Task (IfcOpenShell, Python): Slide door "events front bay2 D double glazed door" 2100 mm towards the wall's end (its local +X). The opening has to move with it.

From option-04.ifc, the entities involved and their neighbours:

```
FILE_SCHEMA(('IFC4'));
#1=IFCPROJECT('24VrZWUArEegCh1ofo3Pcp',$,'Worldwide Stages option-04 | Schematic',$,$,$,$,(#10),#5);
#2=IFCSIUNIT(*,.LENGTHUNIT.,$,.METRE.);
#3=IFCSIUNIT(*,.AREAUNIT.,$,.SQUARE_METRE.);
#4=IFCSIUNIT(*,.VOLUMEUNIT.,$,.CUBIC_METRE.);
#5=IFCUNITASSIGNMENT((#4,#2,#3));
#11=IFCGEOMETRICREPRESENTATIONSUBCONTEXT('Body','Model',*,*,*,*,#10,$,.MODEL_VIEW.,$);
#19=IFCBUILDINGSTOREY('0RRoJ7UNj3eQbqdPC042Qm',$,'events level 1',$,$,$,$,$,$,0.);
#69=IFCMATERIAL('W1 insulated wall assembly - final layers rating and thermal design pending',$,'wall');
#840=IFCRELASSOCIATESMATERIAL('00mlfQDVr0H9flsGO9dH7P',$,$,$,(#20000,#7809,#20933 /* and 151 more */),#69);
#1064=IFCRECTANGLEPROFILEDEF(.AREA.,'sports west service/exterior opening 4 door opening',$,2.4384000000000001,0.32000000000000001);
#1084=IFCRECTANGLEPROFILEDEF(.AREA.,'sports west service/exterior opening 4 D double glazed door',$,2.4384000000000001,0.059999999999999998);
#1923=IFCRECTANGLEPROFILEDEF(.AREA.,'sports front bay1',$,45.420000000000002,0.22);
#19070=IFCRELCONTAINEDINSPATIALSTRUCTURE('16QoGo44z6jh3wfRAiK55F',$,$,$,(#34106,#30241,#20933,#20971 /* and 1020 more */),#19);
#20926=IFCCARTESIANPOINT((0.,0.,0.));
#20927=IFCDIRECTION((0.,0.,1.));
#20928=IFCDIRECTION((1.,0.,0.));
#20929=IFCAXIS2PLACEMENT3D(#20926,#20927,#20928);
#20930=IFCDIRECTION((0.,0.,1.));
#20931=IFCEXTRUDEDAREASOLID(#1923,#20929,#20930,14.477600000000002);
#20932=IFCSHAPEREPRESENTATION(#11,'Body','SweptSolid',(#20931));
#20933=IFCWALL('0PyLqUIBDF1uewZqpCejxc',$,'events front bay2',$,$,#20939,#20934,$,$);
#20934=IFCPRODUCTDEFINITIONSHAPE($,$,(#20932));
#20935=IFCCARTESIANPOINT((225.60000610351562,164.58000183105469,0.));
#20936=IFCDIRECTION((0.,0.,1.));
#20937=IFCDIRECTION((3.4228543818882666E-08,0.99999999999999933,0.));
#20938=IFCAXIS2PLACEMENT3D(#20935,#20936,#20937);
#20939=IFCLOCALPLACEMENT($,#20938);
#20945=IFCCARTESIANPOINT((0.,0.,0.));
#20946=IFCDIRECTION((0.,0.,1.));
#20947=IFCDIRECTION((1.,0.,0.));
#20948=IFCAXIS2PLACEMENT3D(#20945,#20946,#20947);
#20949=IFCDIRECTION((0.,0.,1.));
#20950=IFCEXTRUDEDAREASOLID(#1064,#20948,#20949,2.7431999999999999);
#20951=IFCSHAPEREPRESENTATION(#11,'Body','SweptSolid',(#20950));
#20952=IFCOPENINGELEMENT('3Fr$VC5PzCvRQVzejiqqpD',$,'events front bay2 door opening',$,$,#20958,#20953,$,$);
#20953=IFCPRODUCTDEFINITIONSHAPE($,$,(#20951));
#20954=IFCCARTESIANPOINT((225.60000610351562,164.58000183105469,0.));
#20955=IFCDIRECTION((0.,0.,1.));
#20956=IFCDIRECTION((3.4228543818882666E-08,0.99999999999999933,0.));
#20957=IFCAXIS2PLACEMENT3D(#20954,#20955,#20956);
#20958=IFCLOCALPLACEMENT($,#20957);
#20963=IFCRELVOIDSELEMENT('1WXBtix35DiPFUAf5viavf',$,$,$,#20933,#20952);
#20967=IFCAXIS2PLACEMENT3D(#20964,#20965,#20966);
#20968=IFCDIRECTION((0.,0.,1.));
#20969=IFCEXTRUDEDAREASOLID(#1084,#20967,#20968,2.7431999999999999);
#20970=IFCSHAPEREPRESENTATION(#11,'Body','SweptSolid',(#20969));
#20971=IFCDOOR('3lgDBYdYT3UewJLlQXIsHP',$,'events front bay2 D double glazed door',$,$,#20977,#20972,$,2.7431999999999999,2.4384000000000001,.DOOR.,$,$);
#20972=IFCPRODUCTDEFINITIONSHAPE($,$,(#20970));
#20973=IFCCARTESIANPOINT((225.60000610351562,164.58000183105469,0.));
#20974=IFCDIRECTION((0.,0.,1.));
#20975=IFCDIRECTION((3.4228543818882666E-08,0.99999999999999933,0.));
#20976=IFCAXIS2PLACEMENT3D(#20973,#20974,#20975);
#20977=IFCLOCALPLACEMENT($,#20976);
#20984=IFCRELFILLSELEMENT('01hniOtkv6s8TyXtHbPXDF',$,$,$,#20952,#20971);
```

```python
import ifcopenshell
import ifcopenshell.api.geometry
import ifcopenshell.util.placement
import ifcopenshell.util.unit

model = ifcopenshell.open("option-04.ifc")
unit_scale = ifcopenshell.util.unit.calculate_unit_scale(model)

door = model.by_id(20971)
opening = door.FillsVoids[0].RelatingOpeningElement
wall = opening.VoidsElements[0].RelatingBuildingElement

wall_matrix = ifcopenshell.util.placement.get_local_placement(wall.ObjectPlacement)
shift = wall_matrix[:3, 0] * 2.1 / unit_scale
before = ifcopenshell.util.placement.get_local_placement(door.ObjectPlacement)[:3, 3].copy()

# The door is not placed relative to its opening, so move both.
for product in (opening, door):
    matrix = ifcopenshell.util.placement.get_local_placement(product.ObjectPlacement)
    matrix[:3, 3] += shift
    ifcopenshell.api.geometry.edit_object_placement(model, product=product, matrix=matrix, is_si=False)

after = ifcopenshell.util.placement.get_local_placement(door.ObjectPlacement)[:3, 3]
print("door moved by", (after - before).round(3) + 0.0)

model.write("option-04_updated.ifc")
```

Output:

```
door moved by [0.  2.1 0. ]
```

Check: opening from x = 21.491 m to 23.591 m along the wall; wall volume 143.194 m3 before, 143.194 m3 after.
